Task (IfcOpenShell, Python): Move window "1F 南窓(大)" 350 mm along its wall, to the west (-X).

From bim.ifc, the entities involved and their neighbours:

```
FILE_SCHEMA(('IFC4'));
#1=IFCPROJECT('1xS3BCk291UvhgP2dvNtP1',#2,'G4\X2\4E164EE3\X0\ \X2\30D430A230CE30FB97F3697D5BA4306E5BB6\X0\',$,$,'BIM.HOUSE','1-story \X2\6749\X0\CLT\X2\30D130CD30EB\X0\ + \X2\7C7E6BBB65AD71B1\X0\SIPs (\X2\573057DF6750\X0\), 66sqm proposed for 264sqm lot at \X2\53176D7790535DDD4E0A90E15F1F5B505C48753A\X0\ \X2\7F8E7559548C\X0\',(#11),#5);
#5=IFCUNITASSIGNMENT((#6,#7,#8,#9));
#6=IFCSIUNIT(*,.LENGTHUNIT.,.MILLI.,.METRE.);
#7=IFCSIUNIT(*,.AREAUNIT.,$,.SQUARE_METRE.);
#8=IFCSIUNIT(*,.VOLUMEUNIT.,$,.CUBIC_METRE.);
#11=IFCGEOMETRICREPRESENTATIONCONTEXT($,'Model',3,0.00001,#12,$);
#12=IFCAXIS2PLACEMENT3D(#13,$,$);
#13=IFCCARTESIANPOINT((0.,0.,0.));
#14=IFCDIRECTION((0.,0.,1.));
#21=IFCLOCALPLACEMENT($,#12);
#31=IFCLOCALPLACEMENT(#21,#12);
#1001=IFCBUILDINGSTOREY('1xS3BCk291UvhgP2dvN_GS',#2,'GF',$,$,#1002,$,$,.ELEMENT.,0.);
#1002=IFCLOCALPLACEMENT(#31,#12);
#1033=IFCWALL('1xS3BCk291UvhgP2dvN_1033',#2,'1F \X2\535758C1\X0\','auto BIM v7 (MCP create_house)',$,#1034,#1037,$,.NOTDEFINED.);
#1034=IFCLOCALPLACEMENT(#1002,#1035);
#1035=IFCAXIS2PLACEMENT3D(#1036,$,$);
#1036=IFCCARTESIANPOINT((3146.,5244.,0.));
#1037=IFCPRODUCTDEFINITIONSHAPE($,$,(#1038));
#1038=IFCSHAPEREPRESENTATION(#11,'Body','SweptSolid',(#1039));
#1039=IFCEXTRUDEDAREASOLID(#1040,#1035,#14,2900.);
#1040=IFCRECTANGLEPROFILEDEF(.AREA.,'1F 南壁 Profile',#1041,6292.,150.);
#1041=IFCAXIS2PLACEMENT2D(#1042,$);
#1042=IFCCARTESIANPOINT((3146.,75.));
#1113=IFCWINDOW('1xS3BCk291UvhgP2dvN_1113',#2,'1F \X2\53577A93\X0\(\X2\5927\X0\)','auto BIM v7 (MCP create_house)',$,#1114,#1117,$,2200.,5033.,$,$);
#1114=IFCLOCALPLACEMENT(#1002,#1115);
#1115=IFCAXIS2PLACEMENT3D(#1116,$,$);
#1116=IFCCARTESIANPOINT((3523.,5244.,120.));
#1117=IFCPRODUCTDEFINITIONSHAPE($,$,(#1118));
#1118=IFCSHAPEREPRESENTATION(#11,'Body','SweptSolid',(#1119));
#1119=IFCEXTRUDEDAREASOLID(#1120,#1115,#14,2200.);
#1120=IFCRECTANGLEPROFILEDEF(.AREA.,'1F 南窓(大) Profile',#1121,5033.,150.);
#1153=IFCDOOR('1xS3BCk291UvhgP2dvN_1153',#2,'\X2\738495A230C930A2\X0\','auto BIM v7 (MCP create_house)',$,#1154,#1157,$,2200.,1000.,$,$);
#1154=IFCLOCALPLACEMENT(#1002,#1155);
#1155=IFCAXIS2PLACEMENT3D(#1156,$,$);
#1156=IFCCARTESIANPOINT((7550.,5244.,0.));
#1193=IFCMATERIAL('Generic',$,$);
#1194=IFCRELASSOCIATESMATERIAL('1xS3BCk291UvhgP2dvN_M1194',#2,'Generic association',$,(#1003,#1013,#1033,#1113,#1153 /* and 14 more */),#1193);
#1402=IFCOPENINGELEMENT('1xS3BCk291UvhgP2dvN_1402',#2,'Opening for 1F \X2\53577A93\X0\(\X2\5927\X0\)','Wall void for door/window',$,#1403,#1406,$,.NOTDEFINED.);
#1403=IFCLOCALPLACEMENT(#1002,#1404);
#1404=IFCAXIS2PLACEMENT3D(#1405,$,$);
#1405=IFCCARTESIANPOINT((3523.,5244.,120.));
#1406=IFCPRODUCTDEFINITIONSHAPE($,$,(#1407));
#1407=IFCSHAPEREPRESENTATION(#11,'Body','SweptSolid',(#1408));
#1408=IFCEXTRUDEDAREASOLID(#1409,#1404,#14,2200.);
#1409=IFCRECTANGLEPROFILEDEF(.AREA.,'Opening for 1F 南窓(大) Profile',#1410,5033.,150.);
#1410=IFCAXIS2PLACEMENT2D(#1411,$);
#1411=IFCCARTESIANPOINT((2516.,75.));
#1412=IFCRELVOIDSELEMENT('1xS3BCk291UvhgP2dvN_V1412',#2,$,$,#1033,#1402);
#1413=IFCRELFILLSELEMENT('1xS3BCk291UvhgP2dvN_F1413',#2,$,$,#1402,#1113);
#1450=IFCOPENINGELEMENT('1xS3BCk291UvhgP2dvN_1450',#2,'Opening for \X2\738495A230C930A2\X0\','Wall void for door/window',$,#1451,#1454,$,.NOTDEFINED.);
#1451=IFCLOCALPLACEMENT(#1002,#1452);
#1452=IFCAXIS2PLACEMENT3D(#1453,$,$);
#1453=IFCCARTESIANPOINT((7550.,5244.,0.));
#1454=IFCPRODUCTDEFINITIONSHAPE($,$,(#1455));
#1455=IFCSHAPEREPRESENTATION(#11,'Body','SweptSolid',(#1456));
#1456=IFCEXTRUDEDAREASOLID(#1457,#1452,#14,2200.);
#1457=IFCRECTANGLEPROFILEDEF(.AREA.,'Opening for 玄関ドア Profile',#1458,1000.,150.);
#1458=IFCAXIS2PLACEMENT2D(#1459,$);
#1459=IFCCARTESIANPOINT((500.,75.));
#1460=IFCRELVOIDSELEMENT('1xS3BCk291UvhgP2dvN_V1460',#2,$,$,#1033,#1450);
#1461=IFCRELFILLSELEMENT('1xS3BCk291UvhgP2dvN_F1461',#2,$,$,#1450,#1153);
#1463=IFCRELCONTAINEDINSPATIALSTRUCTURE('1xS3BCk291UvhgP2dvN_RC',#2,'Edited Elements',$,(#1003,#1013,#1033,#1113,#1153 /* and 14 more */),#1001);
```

```python
import ifcopenshell
import ifcopenshell.api.geometry
import ifcopenshell.util.placement
import ifcopenshell.util.unit

model = ifcopenshell.open("bim.ifc")
unit_scale = ifcopenshell.util.unit.calculate_unit_scale(model)

window = model.by_guid("1xS3BCk291UvhgP2dvN_1113")
opening = window.FillsVoids[0].RelatingOpeningElement
wall = opening.VoidsElements[0].RelatingBuildingElement

wall_matrix = ifcopenshell.util.placement.get_local_placement(wall.ObjectPlacement)
shift = wall_matrix[:3, 0] * -0.35 / unit_scale
before = ifcopenshell.util.placement.get_local_placement(window.ObjectPlacement)[:3, 3].copy()

# The window is not placed relative to its opening, so move both.
for product in (opening, window):
    matrix = ifcopenshell.util.placement.get_local_placement(product.ObjectPlacement)
    matrix[:3, 3] += shift
    ifcopenshell.api.geometry.edit_object_placement(model, product=product, matrix=matrix, is_si=False)

after = ifcopenshell.util.placement.get_local_placement(window.ObjectPlacement)[:3, 3]
print("window moved by", (after - before).round(3) + 0.0)

model.write("bim_rev.ifc")
```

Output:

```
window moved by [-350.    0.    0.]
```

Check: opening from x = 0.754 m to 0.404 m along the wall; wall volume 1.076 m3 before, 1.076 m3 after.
